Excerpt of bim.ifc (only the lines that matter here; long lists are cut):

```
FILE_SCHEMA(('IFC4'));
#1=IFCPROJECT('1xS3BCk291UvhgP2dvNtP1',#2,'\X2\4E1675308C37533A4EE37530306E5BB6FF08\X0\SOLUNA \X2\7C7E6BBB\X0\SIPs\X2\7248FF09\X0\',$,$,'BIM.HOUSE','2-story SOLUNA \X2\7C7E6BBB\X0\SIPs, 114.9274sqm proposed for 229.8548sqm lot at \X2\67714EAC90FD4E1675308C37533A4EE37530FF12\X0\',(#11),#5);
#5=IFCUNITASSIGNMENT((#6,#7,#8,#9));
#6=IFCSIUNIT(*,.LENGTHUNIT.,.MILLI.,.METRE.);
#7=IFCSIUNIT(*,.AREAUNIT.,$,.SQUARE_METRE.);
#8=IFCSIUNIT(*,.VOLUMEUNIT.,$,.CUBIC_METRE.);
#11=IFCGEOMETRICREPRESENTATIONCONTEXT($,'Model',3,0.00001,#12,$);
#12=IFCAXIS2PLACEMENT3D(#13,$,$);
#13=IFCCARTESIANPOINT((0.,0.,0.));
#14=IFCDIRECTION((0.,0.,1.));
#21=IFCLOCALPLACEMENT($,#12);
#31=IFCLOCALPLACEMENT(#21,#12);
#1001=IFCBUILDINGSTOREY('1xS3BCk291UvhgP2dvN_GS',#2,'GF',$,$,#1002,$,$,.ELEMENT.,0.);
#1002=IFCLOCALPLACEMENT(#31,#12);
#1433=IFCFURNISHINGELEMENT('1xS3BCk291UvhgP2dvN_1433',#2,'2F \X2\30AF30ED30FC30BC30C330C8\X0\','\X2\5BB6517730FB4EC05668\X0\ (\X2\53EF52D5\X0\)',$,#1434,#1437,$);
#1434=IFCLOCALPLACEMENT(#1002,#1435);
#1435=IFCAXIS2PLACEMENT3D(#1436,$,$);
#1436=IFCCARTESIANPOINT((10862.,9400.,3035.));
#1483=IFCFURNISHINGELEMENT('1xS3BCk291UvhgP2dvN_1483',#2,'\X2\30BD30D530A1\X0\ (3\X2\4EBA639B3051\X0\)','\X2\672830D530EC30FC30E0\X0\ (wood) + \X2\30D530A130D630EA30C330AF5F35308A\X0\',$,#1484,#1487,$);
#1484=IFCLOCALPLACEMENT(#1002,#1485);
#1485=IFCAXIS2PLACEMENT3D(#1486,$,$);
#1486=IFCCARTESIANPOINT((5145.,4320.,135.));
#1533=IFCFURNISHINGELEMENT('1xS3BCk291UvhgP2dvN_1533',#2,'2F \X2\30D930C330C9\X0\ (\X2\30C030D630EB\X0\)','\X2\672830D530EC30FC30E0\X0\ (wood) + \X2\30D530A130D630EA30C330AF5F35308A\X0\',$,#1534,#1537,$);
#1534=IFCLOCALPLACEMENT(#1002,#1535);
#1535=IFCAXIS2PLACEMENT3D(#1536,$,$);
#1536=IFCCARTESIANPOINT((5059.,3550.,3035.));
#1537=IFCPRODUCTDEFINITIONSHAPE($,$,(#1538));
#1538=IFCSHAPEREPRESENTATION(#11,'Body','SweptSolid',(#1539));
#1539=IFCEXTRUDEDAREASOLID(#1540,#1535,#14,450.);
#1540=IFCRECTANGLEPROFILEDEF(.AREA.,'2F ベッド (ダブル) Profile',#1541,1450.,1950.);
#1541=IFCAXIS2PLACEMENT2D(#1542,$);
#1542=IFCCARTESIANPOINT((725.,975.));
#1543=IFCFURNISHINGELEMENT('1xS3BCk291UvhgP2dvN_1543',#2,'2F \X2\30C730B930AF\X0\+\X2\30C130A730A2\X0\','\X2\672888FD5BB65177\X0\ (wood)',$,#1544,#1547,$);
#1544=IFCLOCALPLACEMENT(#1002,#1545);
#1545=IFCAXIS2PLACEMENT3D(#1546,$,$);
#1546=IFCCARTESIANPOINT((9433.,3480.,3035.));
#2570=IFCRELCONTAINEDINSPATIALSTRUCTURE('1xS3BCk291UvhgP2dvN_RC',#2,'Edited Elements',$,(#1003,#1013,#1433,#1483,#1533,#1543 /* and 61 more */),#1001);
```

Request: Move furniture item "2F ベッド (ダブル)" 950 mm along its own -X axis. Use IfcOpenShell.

```python
import ifcopenshell
import ifcopenshell.api.geometry
import ifcopenshell.util.placement
import ifcopenshell.util.unit

model = ifcopenshell.open("bim.ifc")
unit_scale = ifcopenshell.util.unit.calculate_unit_scale(model)

item = model.by_guid("1xS3BCk291UvhgP2dvN_1533")
matrix = ifcopenshell.util.placement.get_local_placement(item.ObjectPlacement)
matrix[:3, 3] -= matrix[:3, 0] * 0.95 / unit_scale
ifcopenshell.api.geometry.edit_object_placement(model, product=item, matrix=matrix, is_si=False)

print(ifcopenshell.util.placement.get_local_placement(item.ObjectPlacement).round(3) + 0.0)

model.write("bim_rev.ifc")
```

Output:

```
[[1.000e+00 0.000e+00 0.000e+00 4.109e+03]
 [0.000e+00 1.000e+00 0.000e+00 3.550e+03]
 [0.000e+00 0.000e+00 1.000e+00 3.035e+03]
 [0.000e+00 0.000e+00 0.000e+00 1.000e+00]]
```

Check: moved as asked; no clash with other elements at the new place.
